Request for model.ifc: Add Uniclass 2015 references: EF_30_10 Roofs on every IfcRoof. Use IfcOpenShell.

First a look at what the model holds.

```python
import ifcopenshell

model = ifcopenshell.open("model.ifc")
print(model.schema)
print("classifications:", [c.Name for c in model.by_type("IfcClassification")])
for ifc_class in ("IfcDoor", "IfcRoof", "IfcStair", "IfcWall", "IfcWindow"):
    print(ifc_class, len(model.by_type(ifc_class)))
```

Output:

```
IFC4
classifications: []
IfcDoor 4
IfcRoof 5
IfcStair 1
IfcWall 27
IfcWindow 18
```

```python
import ifcopenshell
import ifcopenshell.api.classification

model = ifcopenshell.open("model.ifc")

system = ifcopenshell.api.classification.add_classification(model, classification="Uniclass 2015")

codes = {
    "IfcRoof": ("EF_30_10", "Roofs"),
}
for ifc_class, (code, name) in codes.items():
    products = model.by_type(ifc_class)
    ifcopenshell.api.classification.add_reference(
        model, products=products, classification=system, identification=code, name=name
    )
    print(code, len(products))

model.write("model-out.ifc")
```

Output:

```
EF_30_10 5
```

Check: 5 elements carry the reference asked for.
